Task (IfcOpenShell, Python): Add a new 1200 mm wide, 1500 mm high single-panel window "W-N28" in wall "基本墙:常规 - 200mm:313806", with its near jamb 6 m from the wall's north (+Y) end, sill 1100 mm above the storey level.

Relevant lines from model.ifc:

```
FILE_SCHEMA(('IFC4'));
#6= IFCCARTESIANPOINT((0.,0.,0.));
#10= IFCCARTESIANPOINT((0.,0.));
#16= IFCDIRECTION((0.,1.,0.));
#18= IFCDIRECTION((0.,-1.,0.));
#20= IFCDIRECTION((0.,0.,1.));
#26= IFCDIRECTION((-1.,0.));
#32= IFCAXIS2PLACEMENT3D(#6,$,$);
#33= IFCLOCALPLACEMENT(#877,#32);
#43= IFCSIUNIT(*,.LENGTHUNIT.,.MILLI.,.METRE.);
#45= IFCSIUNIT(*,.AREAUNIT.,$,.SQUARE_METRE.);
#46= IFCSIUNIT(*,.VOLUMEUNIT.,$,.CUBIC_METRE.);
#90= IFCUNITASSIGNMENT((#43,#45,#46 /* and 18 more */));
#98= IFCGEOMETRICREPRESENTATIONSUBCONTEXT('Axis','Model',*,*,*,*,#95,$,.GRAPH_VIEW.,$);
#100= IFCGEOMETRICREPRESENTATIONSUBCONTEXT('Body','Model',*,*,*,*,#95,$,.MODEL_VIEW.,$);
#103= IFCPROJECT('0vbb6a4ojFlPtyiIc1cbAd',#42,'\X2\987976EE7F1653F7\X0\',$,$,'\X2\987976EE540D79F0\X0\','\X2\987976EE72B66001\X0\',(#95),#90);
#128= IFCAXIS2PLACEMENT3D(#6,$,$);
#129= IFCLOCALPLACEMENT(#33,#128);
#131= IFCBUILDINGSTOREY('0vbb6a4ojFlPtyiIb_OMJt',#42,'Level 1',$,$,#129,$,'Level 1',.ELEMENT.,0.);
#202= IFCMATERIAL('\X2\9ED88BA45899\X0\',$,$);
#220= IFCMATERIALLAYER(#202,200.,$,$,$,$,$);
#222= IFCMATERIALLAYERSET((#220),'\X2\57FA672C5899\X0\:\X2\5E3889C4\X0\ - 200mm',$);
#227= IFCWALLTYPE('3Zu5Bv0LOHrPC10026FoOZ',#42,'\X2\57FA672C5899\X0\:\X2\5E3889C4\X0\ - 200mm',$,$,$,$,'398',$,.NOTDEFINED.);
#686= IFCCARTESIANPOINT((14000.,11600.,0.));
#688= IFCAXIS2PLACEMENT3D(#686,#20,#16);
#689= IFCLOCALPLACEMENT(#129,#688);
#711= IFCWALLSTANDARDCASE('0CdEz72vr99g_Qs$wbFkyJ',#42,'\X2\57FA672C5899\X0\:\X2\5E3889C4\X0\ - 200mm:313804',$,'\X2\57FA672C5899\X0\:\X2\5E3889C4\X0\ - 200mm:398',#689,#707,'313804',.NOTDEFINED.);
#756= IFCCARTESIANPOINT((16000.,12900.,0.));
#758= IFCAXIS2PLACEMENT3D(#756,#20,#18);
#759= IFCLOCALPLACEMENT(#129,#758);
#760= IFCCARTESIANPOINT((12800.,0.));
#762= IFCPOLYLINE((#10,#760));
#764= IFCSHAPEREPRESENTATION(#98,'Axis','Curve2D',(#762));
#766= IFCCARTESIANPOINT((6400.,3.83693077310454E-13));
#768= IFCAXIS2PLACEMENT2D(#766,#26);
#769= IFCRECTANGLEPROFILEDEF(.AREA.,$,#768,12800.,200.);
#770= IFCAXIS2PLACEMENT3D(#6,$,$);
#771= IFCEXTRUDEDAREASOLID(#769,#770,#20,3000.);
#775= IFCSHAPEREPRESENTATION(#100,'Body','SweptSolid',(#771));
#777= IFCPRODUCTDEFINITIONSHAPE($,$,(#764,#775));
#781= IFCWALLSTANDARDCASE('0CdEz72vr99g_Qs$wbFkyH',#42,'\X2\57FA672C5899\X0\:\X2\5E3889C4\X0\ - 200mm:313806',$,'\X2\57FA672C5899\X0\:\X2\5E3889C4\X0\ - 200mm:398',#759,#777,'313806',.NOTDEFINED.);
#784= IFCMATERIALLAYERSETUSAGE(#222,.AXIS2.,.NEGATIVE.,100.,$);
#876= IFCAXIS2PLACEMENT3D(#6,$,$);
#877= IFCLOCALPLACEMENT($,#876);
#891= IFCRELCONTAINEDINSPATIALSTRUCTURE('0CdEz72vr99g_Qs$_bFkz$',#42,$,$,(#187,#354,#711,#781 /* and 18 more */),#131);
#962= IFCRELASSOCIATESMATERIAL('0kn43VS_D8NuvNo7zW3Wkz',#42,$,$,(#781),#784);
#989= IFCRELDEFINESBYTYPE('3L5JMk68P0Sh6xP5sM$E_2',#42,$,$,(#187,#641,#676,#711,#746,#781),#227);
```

```python
import numpy as np
import ifcopenshell
import ifcopenshell.api.feature
import ifcopenshell.api.geometry
import ifcopenshell.api.root
import ifcopenshell.api.spatial
import ifcopenshell.geom
import ifcopenshell.util.element
import ifcopenshell.util.placement
import ifcopenshell.util.representation
import ifcopenshell.util.shape
import ifcopenshell.util.unit

model = ifcopenshell.open("model.ifc")
unit_scale = ifcopenshell.util.unit.calculate_unit_scale(model)
settings = ifcopenshell.geom.settings()


def volume(element):
    """Net volume in cubic metres, openings subtracted."""
    shape = ifcopenshell.geom.create_shape(settings, element)
    return ifcopenshell.util.shape.get_volume(shape.geometry)


wall = model.by_guid("0CdEz72vr99g_Qs$wbFkyH")
storey = ifcopenshell.util.element.get_container(wall, ifc_class="IfcBuildingStorey")
context = ifcopenshell.util.representation.get_context(model, "Model", "Body", "MODEL_VIEW")
before = volume(wall)

width, height, from_end, sill = 1.2, 1.5, 6, 1.1  # metres

# The wall runs along its own X axis, and the end named is its -X end.
wall_shape = ifcopenshell.geom.create_shape(settings, wall)
x, y, z = ifcopenshell.util.shape.get_vertices(wall_shape.geometry).T
start = x.min() + from_end
face, thickness = float(y.min()), float(y.max() - y.min())
wall_matrix = ifcopenshell.util.placement.get_local_placement(wall.ObjectPlacement)
level = ifcopenshell.util.placement.get_local_placement(storey.ObjectPlacement)[2, 3]


def in_wall(x, y):
    """Placement at x, y metres in the wall's axes, at sill height."""
    matrix = wall_matrix.copy()
    matrix[:, 3] = wall_matrix @ np.array([x / unit_scale, y / unit_scale, 0.0, 1.0])
    matrix[2, 3] = level + sill / unit_scale
    return matrix


# Opening: a box that overshoots both wall faces by 50 mm.
opening = ifcopenshell.api.root.create_entity(model, ifc_class="IfcOpeningElement", predefined_type="OPENING")
box = ifcopenshell.api.geometry.add_wall_representation(
    model, context=context, length=width, height=height, thickness=thickness + 0.1
)
ifcopenshell.api.geometry.assign_representation(model, product=opening, representation=box)
ifcopenshell.api.geometry.edit_object_placement(model, product=opening, matrix=in_wall(start, face - 0.05), is_si=False)
ifcopenshell.api.feature.add_feature(model, feature=opening, element=wall)

window = ifcopenshell.api.root.create_entity(model, ifc_class="IfcWindow", name="W-N28", predefined_type="WINDOW")
window.OverallWidth, window.OverallHeight = width / unit_scale, height / unit_scale
window.PartitioningType = "SINGLE_PANEL"
body = ifcopenshell.api.geometry.add_window_representation(
    model,
    context=context,
    overall_width=window.OverallWidth,
    overall_height=window.OverallHeight,
    partition_type="SINGLE_PANEL",
)
ifcopenshell.api.geometry.assign_representation(model, product=window, representation=body)
ifcopenshell.api.spatial.assign_container(model, products=[window], relating_structure=storey)
ifcopenshell.api.feature.add_filling(model, opening=opening, element=window)

# Centre the window in the wall's thickness.
ifcopenshell.api.geometry.edit_object_placement(model, product=window, matrix=in_wall(start, face), is_si=False)
window_shape = ifcopenshell.geom.create_shape(settings, window)
depth = ifcopenshell.util.shape.get_vertices(window_shape.geometry)[:, 1]
offset = face + thickness / 2 - (depth.min() + depth.max()) / 2
ifcopenshell.api.geometry.edit_object_placement(model, product=window, matrix=in_wall(start, offset), is_si=False)

after = volume(wall)

print(f"wall volume {before:.3f} -> {after:.3f} m3")

model.write("model_edited.ifc")
```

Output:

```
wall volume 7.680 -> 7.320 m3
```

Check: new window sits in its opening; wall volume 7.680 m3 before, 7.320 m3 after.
